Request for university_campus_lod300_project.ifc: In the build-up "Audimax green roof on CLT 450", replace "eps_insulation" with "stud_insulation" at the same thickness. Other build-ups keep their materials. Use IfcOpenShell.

First a look at what the model holds.

```python
import ifcopenshell
import ifcopenshell.util.element

model = ifcopenshell.open("university_campus_lod300_project.ifc")
print(model.schema)
for layer_set in model.by_type("IfcMaterialLayerSet"):
    if layer_set.LayerSetName == "Audimax green roof on CLT 450":
        for layer in layer_set.MaterialLayers:
            print(layer.id(), layer.Material and layer.Material.Name, layer.LayerThickness, sep=" | ")
        print(len(ifcopenshell.util.element.get_elements_by_material(model, layer_set)), "elements and types use it")
print(sorted(m.Name for m in model.by_type("IfcMaterial") if m.Name)[:60])
```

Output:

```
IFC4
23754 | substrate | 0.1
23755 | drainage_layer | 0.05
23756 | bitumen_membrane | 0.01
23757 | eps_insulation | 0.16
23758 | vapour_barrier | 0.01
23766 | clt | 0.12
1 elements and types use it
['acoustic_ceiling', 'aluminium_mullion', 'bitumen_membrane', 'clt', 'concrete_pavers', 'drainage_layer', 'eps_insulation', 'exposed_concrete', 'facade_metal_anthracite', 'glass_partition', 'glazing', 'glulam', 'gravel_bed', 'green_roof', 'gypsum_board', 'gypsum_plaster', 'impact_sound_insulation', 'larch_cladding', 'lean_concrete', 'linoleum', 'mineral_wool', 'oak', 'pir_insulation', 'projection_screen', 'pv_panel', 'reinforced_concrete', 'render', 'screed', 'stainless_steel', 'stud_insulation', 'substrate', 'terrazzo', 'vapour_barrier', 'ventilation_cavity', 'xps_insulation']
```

```python
import ifcopenshell
import ifcopenshell.api.material

model = ifcopenshell.open("university_campus_lod300_project.ifc")

layer_set = next(s for s in model.by_type("IfcMaterialLayerSet") if s.LayerSetName == "Audimax green roof on CLT 450")
layer = next(l for l in layer_set.MaterialLayers if l.Material and l.Material.Name == "eps_insulation")
material = next(m for m in model.by_type("IfcMaterial") if m.Name == "stud_insulation")

# Point this one layer at the other material; renaming the old one would change it everywhere.
ifcopenshell.api.material.edit_layer(model, layer=layer, attributes={"Name": material.Name}, material=material)

print([l.Material.Name if l.Material else None for l in layer_set.MaterialLayers])

model.write("university_campus_lod300_project_edited.ifc")
```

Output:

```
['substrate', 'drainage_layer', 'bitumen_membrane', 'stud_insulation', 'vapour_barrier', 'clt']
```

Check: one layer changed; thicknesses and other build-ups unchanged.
